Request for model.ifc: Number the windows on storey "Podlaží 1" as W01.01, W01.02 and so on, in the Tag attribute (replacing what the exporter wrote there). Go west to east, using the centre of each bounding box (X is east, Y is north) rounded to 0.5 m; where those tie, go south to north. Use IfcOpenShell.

First a look at what the model holds.

```python
import ifcopenshell
import ifcopenshell.util.element
import ifcopenshell.util.placement

model = ifcopenshell.open("model.ifc")
print(model.schema)
storey = next(s for s in model.by_type("IfcBuildingStorey") if s.Name == "Podlaží 1")
windows = [e for e in ifcopenshell.util.element.get_decomposition(storey) if e.is_a("IfcWindow")]
for e in sorted(windows, key=lambda e: e.id()):
    origin = ifcopenshell.util.placement.get_local_placement(e.ObjectPlacement)[:3, 3]
    print(e.id(), e.Tag, e.Name, origin.round(2) + 0.0, sep=" | ")
```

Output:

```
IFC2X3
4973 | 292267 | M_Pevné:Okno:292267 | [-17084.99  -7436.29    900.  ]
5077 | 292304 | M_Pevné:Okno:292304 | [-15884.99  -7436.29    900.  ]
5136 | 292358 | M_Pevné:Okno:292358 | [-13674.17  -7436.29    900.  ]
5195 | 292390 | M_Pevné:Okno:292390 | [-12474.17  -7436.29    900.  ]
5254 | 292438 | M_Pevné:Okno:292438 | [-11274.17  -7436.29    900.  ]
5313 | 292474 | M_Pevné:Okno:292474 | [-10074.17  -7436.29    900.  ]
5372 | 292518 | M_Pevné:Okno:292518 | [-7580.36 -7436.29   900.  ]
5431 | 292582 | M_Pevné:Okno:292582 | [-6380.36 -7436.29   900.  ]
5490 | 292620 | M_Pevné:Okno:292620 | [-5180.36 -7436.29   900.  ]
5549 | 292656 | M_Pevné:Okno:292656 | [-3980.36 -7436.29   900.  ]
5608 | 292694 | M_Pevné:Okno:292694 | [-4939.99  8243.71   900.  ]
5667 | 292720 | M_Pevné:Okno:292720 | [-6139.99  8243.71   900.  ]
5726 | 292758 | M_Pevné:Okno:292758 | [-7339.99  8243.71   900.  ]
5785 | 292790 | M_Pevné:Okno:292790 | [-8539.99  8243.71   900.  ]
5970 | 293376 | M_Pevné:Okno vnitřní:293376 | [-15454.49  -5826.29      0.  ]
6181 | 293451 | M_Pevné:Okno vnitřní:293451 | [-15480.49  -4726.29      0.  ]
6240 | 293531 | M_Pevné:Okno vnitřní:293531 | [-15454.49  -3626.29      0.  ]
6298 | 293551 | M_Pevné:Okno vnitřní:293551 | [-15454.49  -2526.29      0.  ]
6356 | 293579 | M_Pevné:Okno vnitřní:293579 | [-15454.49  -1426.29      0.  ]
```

```python
import ifcopenshell
import ifcopenshell.geom
import ifcopenshell.util.element
import ifcopenshell.util.shape

model = ifcopenshell.open("model.ifc")
settings = ifcopenshell.geom.settings()
settings.set("use-world-coords", True)


def centre(element):
    shape = ifcopenshell.geom.create_shape(settings, element)
    return ifcopenshell.util.shape.get_bbox_centroid(shape.geometry)


storey = next(s for s in model.by_type("IfcBuildingStorey") if s.Name == "Podlaží 1")
windows = [e for e in ifcopenshell.util.element.get_decomposition(storey) if e.is_a("IfcWindow")]

# Insertion points can sit at a corner or the storey origin, so sort by the geometry (in metres).
centres = {e: centre(e) for e in windows}
windows.sort(key=lambda e: (round(centres[e][0] / 0.5), centres[e][1]))

for i, e in enumerate(windows, start=1):
    number = f"W01.{i:02d}"
    e.Tag = number
    print(e.id(), number)

model.write("model_edited.ifc")
```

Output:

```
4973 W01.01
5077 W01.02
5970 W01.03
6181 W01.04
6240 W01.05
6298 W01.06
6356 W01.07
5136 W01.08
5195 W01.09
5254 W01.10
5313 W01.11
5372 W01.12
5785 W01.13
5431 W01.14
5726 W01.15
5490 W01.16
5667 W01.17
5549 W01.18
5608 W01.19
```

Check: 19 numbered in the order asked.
